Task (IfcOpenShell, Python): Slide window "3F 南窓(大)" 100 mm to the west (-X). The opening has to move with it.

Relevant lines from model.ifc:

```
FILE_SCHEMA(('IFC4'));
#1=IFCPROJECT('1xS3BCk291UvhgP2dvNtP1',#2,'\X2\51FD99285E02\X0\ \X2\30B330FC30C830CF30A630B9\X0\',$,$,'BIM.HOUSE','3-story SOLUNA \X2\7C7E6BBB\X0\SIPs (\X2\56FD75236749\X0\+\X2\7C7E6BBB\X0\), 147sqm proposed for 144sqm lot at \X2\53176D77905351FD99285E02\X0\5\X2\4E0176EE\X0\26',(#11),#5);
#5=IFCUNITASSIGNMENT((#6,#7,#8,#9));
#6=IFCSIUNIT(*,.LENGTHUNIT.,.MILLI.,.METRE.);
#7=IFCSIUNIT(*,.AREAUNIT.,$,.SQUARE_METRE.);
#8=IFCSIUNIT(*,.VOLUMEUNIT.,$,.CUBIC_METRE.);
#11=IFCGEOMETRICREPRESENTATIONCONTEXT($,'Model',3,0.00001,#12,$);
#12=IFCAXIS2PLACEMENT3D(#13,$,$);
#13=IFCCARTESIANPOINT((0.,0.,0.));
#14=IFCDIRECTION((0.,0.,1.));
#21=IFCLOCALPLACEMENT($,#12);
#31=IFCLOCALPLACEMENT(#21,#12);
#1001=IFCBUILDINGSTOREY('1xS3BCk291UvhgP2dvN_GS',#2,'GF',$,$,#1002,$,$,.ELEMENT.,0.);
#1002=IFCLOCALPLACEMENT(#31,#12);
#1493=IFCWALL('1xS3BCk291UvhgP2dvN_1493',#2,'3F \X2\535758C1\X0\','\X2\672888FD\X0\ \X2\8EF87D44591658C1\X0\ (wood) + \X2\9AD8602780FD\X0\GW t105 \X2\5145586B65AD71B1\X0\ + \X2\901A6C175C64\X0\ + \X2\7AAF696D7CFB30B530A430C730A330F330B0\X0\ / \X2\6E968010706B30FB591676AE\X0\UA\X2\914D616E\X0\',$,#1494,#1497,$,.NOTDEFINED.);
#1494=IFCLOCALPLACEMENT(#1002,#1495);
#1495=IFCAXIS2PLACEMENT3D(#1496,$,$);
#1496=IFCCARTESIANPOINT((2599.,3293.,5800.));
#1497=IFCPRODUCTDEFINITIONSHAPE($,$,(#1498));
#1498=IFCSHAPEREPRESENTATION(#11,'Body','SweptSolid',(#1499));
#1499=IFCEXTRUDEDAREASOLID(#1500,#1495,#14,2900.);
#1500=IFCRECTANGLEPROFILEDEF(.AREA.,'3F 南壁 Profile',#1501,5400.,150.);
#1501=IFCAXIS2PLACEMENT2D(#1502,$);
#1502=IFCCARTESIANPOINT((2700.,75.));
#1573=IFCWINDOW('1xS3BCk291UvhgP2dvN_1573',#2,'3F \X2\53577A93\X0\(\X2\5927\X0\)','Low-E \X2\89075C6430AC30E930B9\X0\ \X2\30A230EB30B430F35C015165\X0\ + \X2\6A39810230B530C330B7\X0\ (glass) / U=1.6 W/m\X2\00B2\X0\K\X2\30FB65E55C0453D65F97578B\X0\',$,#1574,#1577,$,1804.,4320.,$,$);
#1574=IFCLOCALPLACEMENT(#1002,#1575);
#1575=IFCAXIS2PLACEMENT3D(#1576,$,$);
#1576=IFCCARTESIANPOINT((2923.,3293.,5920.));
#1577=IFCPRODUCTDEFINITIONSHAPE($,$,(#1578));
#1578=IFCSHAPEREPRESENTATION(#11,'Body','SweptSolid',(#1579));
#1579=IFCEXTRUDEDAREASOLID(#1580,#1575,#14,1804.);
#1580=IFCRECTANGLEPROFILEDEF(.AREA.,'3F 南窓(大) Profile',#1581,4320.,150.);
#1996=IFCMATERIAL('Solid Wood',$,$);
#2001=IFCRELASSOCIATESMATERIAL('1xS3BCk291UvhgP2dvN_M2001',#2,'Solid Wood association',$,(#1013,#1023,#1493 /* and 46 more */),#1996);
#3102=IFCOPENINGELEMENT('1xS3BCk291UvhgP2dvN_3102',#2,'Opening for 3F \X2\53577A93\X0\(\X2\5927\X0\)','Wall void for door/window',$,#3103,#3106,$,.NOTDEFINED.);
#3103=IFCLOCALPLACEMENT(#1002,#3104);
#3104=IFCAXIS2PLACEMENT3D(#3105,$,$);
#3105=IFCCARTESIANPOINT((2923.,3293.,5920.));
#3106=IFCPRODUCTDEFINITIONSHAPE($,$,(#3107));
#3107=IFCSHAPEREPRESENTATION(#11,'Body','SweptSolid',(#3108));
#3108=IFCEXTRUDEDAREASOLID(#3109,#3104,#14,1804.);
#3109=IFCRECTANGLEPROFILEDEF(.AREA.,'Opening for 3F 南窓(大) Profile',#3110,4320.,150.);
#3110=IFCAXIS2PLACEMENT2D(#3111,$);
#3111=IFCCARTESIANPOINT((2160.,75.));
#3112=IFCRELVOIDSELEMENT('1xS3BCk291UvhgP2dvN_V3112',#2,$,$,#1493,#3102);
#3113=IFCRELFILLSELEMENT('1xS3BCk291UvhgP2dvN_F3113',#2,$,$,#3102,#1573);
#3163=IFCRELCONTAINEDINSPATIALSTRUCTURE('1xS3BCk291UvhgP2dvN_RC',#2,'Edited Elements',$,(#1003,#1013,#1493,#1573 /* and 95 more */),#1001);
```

```python
import ifcopenshell
import ifcopenshell.api.geometry
import ifcopenshell.util.placement
import ifcopenshell.util.unit

model = ifcopenshell.open("model.ifc")
unit_scale = ifcopenshell.util.unit.calculate_unit_scale(model)

window = model.by_guid("1xS3BCk291UvhgP2dvN_1573")
opening = window.FillsVoids[0].RelatingOpeningElement
wall = opening.VoidsElements[0].RelatingBuildingElement

wall_matrix = ifcopenshell.util.placement.get_local_placement(wall.ObjectPlacement)
shift = wall_matrix[:3, 0] * -0.1 / unit_scale
before = ifcopenshell.util.placement.get_local_placement(window.ObjectPlacement)[:3, 3].copy()

# The window is not placed relative to its opening, so move both.
for product in (opening, window):
    matrix = ifcopenshell.util.placement.get_local_placement(product.ObjectPlacement)
    matrix[:3, 3] += shift
    ifcopenshell.api.geometry.edit_object_placement(model, product=product, matrix=matrix, is_si=False)

after = ifcopenshell.util.placement.get_local_placement(window.ObjectPlacement)[:3, 3]
print("window moved by", (after - before).round(3) + 0.0)

model.write("model_rev.ifc")
```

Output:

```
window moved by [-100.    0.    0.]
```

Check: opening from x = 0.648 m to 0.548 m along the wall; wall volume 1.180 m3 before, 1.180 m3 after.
